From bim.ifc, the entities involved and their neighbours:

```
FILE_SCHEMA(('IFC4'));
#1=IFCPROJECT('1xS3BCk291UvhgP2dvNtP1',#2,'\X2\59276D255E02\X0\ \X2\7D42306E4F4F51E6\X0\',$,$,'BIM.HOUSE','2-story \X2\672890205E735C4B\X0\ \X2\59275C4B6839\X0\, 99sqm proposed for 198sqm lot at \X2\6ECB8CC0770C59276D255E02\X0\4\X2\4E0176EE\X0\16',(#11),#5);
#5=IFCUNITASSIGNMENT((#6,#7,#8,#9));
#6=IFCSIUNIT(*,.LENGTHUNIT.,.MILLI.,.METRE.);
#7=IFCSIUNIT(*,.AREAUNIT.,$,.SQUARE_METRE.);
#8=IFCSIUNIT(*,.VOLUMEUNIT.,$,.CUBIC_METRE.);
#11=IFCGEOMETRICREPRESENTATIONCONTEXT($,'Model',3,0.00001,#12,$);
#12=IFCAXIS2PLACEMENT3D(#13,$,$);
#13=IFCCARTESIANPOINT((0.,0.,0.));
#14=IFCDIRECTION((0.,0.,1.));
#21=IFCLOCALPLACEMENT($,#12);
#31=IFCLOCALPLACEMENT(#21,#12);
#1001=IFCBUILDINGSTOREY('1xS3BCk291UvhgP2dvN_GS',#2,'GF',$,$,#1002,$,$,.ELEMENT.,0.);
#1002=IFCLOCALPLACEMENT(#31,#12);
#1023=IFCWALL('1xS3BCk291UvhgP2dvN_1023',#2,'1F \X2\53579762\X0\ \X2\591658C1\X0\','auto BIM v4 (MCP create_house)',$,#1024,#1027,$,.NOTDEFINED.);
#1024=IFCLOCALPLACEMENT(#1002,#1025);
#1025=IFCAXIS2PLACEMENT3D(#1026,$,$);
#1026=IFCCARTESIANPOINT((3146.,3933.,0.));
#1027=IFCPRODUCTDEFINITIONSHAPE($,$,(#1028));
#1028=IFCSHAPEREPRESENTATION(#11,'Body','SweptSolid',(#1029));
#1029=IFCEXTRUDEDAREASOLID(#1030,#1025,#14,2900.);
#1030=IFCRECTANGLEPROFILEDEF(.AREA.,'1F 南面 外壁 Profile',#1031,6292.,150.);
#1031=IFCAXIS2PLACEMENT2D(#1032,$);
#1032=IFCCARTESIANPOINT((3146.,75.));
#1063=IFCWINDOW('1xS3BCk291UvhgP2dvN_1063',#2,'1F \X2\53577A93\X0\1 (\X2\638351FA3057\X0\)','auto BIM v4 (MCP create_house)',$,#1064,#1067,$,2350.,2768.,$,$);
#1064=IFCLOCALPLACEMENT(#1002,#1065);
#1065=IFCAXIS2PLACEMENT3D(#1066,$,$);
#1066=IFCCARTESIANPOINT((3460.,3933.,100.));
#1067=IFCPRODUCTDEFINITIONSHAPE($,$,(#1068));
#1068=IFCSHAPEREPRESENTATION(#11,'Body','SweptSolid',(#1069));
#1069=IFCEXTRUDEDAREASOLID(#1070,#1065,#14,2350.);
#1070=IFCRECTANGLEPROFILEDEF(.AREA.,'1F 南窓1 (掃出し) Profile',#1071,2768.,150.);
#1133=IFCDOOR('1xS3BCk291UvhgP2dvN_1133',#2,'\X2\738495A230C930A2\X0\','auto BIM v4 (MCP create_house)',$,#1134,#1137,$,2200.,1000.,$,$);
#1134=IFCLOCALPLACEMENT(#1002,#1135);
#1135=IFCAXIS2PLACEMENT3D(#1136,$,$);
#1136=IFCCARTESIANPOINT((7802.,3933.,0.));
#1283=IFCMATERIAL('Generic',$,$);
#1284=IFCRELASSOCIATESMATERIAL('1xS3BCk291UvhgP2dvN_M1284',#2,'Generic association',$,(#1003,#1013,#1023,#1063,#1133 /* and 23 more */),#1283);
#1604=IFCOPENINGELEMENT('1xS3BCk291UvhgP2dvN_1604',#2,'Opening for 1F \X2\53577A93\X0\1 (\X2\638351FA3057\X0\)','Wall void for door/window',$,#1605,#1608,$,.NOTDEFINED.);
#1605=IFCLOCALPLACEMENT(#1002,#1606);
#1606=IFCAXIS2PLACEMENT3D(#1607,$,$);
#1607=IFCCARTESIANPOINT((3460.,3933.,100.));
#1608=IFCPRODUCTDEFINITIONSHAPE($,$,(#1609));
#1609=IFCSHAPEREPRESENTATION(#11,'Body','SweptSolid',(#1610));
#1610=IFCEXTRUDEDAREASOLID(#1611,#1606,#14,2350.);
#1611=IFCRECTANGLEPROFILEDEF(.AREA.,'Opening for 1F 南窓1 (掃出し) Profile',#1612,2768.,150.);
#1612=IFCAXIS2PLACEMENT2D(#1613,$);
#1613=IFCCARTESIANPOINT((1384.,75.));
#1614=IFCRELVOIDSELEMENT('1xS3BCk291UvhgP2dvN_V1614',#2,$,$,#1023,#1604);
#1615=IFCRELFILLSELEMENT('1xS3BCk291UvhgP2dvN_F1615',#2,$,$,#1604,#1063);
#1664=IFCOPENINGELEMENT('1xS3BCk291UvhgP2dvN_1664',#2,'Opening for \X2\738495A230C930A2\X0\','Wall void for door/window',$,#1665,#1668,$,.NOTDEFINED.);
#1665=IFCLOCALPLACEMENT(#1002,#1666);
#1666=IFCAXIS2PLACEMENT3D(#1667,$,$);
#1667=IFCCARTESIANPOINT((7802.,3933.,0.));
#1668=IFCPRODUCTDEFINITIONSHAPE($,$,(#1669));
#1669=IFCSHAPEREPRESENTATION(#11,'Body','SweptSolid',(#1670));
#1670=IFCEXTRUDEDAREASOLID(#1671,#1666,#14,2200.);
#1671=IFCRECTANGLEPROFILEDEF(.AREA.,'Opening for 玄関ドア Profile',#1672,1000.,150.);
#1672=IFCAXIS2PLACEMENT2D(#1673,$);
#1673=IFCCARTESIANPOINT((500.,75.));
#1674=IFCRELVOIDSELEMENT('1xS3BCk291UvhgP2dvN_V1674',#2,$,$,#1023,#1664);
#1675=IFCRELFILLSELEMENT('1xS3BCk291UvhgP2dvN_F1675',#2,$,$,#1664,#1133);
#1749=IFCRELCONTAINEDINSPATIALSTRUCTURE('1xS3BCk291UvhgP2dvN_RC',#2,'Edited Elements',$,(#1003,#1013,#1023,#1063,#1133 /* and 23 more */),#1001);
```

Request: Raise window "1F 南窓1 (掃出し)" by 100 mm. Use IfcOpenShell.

```python
import numpy as np
import ifcopenshell
import ifcopenshell.api.geometry
import ifcopenshell.util.placement
import ifcopenshell.util.unit

model = ifcopenshell.open("bim.ifc")
unit_scale = ifcopenshell.util.unit.calculate_unit_scale(model)

window = model.by_guid("1xS3BCk291UvhgP2dvN_1063")
opening = window.FillsVoids[0].RelatingOpeningElement
dz = 100.0

shift = np.array([0.0, 0.0, dz])
# The window is not placed relative to its opening, so move both.
for product in (opening, window):
    matrix = ifcopenshell.util.placement.get_local_placement(product.ObjectPlacement)
    matrix[:3, 3] += shift
    ifcopenshell.api.geometry.edit_object_placement(model, product=product, matrix=matrix, is_si=False)

print(f"moved by {dz * unit_scale:+.3f} m")

model.write("bim_rev.ifc")
```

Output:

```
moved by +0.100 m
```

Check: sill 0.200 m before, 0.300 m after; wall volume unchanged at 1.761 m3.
